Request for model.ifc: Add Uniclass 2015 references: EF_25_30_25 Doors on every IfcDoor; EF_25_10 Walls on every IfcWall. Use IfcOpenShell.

First a look at what the model holds.

```python
import ifcopenshell

model = ifcopenshell.open("model.ifc")
print(model.schema)
print("classifications:", [c.Name for c in model.by_type("IfcClassification")])
for ifc_class in ("IfcDoor", "IfcRoof", "IfcStair", "IfcWall", "IfcWindow"):
    print(ifc_class, len(model.by_type(ifc_class)))
```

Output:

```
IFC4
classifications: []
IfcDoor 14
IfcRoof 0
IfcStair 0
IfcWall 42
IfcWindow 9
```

```python
import ifcopenshell
import ifcopenshell.api.classification

model = ifcopenshell.open("model.ifc")

system = ifcopenshell.api.classification.add_classification(model, classification="Uniclass 2015")

codes = {
    "IfcDoor": ("EF_25_30_25", "Doors"),
    "IfcWall": ("EF_25_10", "Walls"),
}
for ifc_class, (code, name) in codes.items():
    products = model.by_type(ifc_class)
    ifcopenshell.api.classification.add_reference(
        model, products=products, classification=system, identification=code, name=name
    )
    print(code, len(products))

model.write("model_edited.ifc")
```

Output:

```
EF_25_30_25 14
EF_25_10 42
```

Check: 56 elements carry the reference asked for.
